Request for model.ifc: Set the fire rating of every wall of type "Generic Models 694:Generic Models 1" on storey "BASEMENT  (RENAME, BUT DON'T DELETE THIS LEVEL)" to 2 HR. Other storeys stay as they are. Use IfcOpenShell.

First a look at what the model holds.

```python
import ifcopenshell
import ifcopenshell.util.element

model = ifcopenshell.open("model.ifc")
print(model.schema)
storey = next(s for s in model.by_type("IfcBuildingStorey") if s.Name == "BASEMENT  (RENAME, BUT DON'T DELETE THIS LEVEL)")
walls = [e for e in ifcopenshell.util.element.get_decomposition(storey) if e.is_a("IfcWall")]
seen = {}
for e in walls:
    element_type = ifcopenshell.util.element.get_type(e)
    key = (element_type.Name if element_type != e and element_type else None, ifcopenshell.util.element.get_pset(e, "Pset_WallCommon", "FireRating"))
    seen[key] = seen.get(key, 0) + 1
for (name, value), count in sorted(seen.items(), key=str):
    print(count, "x", name, "|", value)
```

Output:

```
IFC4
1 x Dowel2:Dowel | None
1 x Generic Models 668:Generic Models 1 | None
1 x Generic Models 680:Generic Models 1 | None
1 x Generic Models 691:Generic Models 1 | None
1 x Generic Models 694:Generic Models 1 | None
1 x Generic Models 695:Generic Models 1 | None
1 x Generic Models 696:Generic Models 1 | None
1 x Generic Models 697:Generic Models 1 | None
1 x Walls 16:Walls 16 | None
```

```python
import ifcopenshell
import ifcopenshell.api.pset
import ifcopenshell.util.element

model = ifcopenshell.open("model.ifc")

storey = next(s for s in model.by_type("IfcBuildingStorey") if s.Name == "BASEMENT  (RENAME, BUT DON'T DELETE THIS LEVEL)")
walls = [e for e in ifcopenshell.util.element.get_decomposition(storey) if e.is_a("IfcWall")]

count = 0
for e in walls:
    element_type = ifcopenshell.util.element.get_type(e)
    if element_type in (None, e) or element_type.Name != "Generic Models 694:Generic Models 1":
        continue
    # add_pset returns the element's existing set when there is one.
    pset = ifcopenshell.api.pset.add_pset(model, product=e, name="Pset_WallCommon")
    ifcopenshell.api.pset.edit_pset(model, pset=pset, properties={"FireRating": "2 HR"})
    count += 1

print(count, "walls updated")

model.write("model_updated.ifc")
```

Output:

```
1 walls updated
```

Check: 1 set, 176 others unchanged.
